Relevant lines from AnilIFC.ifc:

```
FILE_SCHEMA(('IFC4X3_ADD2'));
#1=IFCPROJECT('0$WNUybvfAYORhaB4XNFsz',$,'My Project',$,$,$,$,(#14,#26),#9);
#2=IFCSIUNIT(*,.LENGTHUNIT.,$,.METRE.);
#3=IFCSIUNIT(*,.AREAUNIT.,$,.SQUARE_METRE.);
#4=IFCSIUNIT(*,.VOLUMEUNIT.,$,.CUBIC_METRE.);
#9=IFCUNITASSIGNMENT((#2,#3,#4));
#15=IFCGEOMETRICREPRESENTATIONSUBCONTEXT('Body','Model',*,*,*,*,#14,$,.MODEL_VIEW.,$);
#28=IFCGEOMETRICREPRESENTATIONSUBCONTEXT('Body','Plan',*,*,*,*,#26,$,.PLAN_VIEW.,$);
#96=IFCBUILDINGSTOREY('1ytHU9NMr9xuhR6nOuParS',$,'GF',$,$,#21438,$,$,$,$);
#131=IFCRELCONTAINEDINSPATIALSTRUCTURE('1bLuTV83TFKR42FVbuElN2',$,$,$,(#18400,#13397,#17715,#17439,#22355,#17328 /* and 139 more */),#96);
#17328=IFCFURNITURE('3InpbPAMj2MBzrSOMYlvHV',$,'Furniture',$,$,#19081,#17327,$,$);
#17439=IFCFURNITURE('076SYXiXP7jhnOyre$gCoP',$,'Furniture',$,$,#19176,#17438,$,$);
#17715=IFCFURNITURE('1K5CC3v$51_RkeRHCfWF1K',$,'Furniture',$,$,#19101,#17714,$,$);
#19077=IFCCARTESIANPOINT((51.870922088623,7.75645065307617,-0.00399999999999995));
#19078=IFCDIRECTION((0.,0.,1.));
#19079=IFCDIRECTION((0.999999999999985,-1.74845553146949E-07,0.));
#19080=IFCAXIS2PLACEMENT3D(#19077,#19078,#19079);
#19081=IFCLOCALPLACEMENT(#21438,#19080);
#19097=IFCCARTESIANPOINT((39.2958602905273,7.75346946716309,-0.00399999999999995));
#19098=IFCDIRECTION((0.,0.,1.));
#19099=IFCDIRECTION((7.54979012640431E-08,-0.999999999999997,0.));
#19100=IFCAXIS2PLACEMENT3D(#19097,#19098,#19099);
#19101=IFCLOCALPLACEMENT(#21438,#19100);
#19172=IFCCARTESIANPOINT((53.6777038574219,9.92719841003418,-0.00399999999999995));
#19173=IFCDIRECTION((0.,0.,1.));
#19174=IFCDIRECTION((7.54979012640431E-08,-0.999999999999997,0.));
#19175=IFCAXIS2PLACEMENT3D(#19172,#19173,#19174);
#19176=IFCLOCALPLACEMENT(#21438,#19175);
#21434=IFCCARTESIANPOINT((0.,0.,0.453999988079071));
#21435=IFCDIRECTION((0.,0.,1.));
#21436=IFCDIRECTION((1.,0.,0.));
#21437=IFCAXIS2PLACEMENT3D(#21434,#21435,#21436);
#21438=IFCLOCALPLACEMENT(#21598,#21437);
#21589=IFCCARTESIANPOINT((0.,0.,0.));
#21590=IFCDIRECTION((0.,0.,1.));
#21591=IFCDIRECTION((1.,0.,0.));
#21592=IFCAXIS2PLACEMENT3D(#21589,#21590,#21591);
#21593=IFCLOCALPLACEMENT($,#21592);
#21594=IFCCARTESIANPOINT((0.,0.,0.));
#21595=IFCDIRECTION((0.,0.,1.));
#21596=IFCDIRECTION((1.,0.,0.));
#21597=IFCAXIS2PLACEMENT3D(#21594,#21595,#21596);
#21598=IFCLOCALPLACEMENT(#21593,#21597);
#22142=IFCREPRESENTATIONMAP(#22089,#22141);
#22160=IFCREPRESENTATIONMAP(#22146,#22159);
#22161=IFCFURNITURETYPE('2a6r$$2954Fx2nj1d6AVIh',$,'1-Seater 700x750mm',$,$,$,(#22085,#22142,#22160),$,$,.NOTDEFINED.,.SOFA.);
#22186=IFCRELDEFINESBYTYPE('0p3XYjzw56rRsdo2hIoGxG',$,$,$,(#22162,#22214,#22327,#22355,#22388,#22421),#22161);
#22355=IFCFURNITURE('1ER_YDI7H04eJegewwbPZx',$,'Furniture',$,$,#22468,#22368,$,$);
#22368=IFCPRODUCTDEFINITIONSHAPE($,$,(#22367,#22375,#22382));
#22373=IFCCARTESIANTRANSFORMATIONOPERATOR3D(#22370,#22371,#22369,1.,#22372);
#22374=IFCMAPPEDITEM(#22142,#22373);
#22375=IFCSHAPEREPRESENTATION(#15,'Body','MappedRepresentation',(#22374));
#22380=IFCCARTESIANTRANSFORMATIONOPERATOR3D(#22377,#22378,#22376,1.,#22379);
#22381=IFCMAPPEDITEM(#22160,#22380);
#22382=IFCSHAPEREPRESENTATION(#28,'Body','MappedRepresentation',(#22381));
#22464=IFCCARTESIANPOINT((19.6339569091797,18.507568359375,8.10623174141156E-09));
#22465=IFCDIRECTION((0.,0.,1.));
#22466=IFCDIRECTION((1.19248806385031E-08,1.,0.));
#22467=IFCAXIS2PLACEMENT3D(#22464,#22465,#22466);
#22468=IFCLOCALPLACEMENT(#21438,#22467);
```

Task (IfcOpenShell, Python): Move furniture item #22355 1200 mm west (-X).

```python
import ifcopenshell
import ifcopenshell.api.geometry
import ifcopenshell.util.placement

model = ifcopenshell.open("AnilIFC.ifc")

item = model.by_guid("1ER_YDI7H04eJegewwbPZx")
matrix = ifcopenshell.util.placement.get_local_placement(item.ObjectPlacement)
matrix[0, 3] -= 1.2
ifcopenshell.api.geometry.edit_object_placement(model, product=item, matrix=matrix, is_si=False)

print(ifcopenshell.util.placement.get_local_placement(item.ObjectPlacement).round(3) + 0.0)

model.write("AnilIFC_edited.ifc")
```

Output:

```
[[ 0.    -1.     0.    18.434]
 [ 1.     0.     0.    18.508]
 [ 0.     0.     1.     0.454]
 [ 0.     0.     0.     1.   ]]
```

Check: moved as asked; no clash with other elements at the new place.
